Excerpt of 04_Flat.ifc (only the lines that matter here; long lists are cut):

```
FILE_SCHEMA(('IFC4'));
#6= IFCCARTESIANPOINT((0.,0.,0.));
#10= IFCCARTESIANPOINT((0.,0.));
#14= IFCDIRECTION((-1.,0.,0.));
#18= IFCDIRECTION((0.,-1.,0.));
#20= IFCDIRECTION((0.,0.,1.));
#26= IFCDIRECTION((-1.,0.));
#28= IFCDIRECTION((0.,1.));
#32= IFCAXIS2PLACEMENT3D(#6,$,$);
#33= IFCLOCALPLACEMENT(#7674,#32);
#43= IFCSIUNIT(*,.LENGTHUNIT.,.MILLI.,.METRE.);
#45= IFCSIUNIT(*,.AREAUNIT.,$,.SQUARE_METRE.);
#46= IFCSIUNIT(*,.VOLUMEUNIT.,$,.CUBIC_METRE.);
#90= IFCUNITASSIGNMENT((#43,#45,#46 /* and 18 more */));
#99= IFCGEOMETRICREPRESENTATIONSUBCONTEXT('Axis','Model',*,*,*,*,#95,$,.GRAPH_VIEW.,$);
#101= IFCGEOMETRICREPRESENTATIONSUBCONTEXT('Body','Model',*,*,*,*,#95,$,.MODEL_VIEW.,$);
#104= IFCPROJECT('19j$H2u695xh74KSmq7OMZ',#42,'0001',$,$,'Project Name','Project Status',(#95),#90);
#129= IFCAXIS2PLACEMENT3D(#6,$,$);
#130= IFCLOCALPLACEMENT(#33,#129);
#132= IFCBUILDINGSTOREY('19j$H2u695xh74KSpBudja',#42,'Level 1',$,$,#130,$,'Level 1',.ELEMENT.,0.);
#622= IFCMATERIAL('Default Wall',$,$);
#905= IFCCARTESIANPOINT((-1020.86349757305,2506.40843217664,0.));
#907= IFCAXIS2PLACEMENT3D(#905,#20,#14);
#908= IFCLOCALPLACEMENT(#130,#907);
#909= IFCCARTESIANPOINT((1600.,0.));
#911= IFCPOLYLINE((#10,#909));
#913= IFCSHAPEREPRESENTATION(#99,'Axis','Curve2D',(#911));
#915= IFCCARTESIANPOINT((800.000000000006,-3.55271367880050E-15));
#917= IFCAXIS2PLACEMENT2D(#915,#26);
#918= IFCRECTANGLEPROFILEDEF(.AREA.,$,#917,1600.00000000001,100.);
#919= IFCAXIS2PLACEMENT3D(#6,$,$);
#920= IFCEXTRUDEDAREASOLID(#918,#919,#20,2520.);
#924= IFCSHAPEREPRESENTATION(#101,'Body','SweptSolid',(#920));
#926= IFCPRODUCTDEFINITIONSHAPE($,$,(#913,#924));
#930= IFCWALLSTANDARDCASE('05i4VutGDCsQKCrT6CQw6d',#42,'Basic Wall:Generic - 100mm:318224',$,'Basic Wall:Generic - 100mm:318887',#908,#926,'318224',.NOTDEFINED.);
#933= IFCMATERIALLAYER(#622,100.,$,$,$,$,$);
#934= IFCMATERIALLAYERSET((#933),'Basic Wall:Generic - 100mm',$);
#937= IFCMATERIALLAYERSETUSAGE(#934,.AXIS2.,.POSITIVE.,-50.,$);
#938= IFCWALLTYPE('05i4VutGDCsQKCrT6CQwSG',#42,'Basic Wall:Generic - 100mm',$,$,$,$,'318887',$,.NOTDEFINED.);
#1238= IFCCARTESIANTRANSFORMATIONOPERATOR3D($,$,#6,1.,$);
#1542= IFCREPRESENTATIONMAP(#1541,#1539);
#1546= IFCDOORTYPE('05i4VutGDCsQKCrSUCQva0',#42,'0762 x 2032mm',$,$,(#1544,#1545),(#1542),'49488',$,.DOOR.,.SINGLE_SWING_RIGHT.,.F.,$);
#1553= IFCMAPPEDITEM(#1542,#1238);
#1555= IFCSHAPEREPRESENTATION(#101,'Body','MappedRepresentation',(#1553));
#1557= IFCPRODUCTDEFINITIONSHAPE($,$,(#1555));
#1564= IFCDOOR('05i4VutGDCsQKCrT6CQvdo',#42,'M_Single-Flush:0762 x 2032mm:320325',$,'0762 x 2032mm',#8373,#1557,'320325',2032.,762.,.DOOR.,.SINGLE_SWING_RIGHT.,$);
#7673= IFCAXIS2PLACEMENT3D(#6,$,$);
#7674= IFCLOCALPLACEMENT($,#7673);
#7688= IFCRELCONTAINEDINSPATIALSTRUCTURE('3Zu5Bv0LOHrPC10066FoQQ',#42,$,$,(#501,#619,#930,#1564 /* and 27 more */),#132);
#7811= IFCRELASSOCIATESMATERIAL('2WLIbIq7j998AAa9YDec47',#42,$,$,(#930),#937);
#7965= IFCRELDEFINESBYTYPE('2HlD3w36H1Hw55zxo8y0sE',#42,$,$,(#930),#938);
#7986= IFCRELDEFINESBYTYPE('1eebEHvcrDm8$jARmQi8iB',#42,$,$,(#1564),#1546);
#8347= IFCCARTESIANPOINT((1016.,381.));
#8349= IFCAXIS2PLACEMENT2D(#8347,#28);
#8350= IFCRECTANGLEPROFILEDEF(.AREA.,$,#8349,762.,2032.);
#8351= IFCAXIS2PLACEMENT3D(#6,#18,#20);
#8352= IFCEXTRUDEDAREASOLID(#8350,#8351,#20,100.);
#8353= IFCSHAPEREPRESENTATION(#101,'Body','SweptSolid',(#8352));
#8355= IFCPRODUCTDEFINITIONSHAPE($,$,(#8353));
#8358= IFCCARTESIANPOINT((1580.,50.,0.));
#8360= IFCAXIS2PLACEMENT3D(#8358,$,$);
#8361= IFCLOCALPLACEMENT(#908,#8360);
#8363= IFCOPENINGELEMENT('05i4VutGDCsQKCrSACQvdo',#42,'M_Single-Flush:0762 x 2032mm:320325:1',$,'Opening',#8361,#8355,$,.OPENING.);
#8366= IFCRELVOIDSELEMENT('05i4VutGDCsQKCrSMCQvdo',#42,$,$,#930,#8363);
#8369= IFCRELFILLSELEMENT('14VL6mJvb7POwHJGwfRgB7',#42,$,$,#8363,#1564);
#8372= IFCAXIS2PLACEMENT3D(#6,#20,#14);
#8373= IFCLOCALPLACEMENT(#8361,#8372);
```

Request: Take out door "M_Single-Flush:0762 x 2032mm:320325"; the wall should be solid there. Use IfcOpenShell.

```python
import ifcopenshell
import ifcopenshell.api.feature
import ifcopenshell.api.root
import ifcopenshell.geom
import ifcopenshell.util.shape

model = ifcopenshell.open("04_Flat.ifc")
settings = ifcopenshell.geom.settings()


def volume(element):
    """Net volume in cubic metres, openings subtracted."""
    shape = ifcopenshell.geom.create_shape(settings, element)
    return ifcopenshell.util.shape.get_volume(shape.geometry)


door = model.by_id(1564)
opening = door.FillsVoids[0].RelatingOpeningElement
wall = opening.VoidsElements[0].RelatingBuildingElement
before = volume(wall)

ifcopenshell.api.root.remove_product(model, product=door)
ifcopenshell.api.feature.remove_feature(model, feature=opening)

after = volume(wall)

print(f"wall volume {before:.3f} -> {after:.3f} m3")

model.write("04_Flat_edited.ifc")
```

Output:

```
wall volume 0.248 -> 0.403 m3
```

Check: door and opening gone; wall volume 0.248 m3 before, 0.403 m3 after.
